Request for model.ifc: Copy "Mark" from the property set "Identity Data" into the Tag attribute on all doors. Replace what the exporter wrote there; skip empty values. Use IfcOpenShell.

First a look at what the model holds.

```python
import ifcopenshell
import ifcopenshell.util.element

model = ifcopenshell.open("model.ifc")
print(model.schema)
doors = model.by_type("IfcDoor")
print(len(doors), "doors")
for e in doors[:8]:
    source = ifcopenshell.util.element.get_pset(e, "Identity Data", "Mark")
    target = e.Tag
    print(e.id(), repr(source), repr(target), sep=" | ")
```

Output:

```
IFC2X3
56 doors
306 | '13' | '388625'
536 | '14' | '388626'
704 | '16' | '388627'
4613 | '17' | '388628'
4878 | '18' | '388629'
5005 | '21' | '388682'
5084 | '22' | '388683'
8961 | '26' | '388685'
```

```python
import ifcopenshell
import ifcopenshell.util.element

model = ifcopenshell.open("model.ifc")

count = 0
for e in model.by_type("IfcDoor"):
    value = ifcopenshell.util.element.get_pset(e, "Identity Data", "Mark")
    current = e.Tag
    if not value or not value.strip() or current == value:
        continue
    e.Tag = value
    count += 1

print(count, "doors updated")

model.write("model_rev.ifc")
```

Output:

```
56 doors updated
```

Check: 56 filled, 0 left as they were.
